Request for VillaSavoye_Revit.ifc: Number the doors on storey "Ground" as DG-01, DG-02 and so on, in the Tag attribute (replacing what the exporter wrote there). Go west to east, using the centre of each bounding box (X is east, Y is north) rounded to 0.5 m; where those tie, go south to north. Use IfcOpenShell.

First a look at what the model holds.

```python
import ifcopenshell
import ifcopenshell.util.element
import ifcopenshell.util.placement

model = ifcopenshell.open("VillaSavoye_Revit.ifc")
print(model.schema)
storey = next(s for s in model.by_type("IfcBuildingStorey") if s.Name == "Ground")
doors = [e for e in ifcopenshell.util.element.get_decomposition(storey) if e.is_a("IfcDoor")]
for e in sorted(doors, key=lambda e: e.id()):
    origin = ifcopenshell.util.placement.get_local_placement(e.ObjectPlacement)[:3, 3]
    print(e.id(), e.Tag, e.Name, origin.round(2) + 0.0, sep=" | ")
```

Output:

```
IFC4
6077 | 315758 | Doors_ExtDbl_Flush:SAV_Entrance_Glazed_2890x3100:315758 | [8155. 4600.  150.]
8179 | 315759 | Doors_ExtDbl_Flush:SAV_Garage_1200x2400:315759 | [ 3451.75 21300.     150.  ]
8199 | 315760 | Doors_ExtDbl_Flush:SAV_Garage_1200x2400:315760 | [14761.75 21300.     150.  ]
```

```python
import ifcopenshell
import ifcopenshell.geom
import ifcopenshell.util.element
import ifcopenshell.util.shape

model = ifcopenshell.open("VillaSavoye_Revit.ifc")
settings = ifcopenshell.geom.settings()
settings.set("use-world-coords", True)


def centre(element):
    shape = ifcopenshell.geom.create_shape(settings, element)
    return ifcopenshell.util.shape.get_bbox_centroid(shape.geometry)


storey = next(s for s in model.by_type("IfcBuildingStorey") if s.Name == "Ground")
doors = [e for e in ifcopenshell.util.element.get_decomposition(storey) if e.is_a("IfcDoor")]

# Insertion points can sit at a corner or the storey origin, so sort by the geometry (in metres).
centres = {e: centre(e) for e in doors}
doors.sort(key=lambda e: (round(centres[e][0] / 0.5), centres[e][1]))

for i, e in enumerate(doors, start=1):
    number = f"DG-{i:02d}"
    e.Tag = number
    print(e.id(), number)

model.write("VillaSavoye_Revit_v2.ifc")
```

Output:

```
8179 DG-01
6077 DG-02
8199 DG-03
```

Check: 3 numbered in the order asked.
